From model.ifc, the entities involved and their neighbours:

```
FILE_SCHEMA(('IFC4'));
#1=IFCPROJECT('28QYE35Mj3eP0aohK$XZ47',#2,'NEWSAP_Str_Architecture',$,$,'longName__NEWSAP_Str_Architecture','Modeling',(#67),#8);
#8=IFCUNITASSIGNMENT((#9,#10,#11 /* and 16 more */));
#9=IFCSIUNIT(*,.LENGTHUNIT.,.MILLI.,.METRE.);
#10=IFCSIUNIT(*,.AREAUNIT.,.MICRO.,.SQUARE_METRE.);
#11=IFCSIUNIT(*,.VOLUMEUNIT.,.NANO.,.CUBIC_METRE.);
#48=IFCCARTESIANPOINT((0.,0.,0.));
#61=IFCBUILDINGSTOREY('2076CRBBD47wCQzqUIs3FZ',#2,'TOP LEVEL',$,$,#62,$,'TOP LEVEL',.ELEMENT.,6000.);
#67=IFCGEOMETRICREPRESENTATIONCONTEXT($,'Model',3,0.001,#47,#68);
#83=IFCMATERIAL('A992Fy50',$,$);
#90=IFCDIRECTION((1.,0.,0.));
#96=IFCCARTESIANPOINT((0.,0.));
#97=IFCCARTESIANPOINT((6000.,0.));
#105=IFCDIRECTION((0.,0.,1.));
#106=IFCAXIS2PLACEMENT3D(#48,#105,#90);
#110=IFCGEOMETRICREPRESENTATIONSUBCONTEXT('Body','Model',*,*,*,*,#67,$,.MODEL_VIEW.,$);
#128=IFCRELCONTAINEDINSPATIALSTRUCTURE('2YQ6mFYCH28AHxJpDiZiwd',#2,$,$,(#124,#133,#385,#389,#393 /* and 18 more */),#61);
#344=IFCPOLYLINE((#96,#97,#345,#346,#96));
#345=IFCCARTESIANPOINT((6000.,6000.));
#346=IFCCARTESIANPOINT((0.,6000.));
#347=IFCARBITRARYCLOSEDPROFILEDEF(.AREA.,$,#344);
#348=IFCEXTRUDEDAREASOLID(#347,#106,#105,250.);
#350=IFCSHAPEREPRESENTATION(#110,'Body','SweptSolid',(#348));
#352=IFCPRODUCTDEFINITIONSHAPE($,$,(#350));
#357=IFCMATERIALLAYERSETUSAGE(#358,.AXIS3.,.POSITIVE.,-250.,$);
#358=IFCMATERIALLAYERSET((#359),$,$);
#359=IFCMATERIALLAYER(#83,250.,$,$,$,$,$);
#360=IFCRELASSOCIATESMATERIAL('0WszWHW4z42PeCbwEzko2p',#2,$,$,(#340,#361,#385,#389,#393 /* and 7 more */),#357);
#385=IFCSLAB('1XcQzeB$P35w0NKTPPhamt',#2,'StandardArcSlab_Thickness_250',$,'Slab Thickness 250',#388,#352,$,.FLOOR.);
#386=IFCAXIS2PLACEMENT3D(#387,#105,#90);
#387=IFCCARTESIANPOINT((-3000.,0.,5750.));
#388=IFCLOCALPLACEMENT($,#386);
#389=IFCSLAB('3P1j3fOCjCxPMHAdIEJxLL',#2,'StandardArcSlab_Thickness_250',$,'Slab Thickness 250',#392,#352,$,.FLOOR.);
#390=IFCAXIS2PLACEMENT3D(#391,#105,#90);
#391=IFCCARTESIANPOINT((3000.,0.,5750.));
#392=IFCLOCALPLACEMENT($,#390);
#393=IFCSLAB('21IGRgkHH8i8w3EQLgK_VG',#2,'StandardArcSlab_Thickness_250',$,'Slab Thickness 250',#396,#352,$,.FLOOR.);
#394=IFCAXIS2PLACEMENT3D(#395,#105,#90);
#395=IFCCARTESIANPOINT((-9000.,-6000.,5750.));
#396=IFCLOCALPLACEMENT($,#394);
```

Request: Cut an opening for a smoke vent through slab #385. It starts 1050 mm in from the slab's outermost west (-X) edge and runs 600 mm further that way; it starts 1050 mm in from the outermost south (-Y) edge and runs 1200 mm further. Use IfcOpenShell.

```python
import numpy as np
import ifcopenshell
import ifcopenshell.api.feature
import ifcopenshell.api.geometry
import ifcopenshell.api.root
import ifcopenshell.geom
import ifcopenshell.util.placement
import ifcopenshell.util.representation
import ifcopenshell.util.shape
import ifcopenshell.util.unit

model = ifcopenshell.open("model.ifc")
unit_scale = ifcopenshell.util.unit.calculate_unit_scale(model)
settings = ifcopenshell.geom.settings()


def volume(element):
    """Net volume in cubic metres, openings subtracted."""
    shape = ifcopenshell.geom.create_shape(settings, element)
    return ifcopenshell.util.shape.get_volume(shape.geometry)


slab = model.by_id(385)
before = volume(slab)

# Extent in the slab's own axes, in metres. The edges named are its -X and -Y sides.
slab_shape = ifcopenshell.geom.create_shape(settings, slab)
vertices = ifcopenshell.util.shape.get_vertices(slab_shape.geometry)
x_min, y_min, bottom = vertices.min(axis=0)
top = vertices[:, 2].max()

opening = ifcopenshell.api.root.create_entity(model, ifc_class="IfcOpeningElement", name="Smoke vent opening", predefined_type="OPENING")
context = ifcopenshell.util.representation.get_context(model, "Model", "Body", "MODEL_VIEW")
width, depth = 0.6, 1.2
outline = [(0.0, 0.0), (width, 0.0), (width, depth), (0.0, depth), (0.0, 0.0)]
# Overshoot both faces by 50 mm so the cut is clean.
shape = ifcopenshell.api.geometry.add_slab_representation(
    model, context=context, depth=top - bottom + 0.1, polyline=outline
)
ifcopenshell.api.geometry.assign_representation(model, product=opening, representation=shape)

matrix = ifcopenshell.util.placement.get_local_placement(slab.ObjectPlacement)
matrix[:, 3] = matrix @ np.append(np.array([x_min + 1.05, y_min + 1.05, bottom - 0.05]) / unit_scale, 1.0)
ifcopenshell.api.geometry.edit_object_placement(model, product=opening, matrix=matrix, is_si=False)
ifcopenshell.api.feature.add_feature(model, feature=opening, element=slab)

after = volume(slab)

print(f"slab volume {before:.3f} -> {after:.3f} m3")

model.write("model_edited.ifc")
```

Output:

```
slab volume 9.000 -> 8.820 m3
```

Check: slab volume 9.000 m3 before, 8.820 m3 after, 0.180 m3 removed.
